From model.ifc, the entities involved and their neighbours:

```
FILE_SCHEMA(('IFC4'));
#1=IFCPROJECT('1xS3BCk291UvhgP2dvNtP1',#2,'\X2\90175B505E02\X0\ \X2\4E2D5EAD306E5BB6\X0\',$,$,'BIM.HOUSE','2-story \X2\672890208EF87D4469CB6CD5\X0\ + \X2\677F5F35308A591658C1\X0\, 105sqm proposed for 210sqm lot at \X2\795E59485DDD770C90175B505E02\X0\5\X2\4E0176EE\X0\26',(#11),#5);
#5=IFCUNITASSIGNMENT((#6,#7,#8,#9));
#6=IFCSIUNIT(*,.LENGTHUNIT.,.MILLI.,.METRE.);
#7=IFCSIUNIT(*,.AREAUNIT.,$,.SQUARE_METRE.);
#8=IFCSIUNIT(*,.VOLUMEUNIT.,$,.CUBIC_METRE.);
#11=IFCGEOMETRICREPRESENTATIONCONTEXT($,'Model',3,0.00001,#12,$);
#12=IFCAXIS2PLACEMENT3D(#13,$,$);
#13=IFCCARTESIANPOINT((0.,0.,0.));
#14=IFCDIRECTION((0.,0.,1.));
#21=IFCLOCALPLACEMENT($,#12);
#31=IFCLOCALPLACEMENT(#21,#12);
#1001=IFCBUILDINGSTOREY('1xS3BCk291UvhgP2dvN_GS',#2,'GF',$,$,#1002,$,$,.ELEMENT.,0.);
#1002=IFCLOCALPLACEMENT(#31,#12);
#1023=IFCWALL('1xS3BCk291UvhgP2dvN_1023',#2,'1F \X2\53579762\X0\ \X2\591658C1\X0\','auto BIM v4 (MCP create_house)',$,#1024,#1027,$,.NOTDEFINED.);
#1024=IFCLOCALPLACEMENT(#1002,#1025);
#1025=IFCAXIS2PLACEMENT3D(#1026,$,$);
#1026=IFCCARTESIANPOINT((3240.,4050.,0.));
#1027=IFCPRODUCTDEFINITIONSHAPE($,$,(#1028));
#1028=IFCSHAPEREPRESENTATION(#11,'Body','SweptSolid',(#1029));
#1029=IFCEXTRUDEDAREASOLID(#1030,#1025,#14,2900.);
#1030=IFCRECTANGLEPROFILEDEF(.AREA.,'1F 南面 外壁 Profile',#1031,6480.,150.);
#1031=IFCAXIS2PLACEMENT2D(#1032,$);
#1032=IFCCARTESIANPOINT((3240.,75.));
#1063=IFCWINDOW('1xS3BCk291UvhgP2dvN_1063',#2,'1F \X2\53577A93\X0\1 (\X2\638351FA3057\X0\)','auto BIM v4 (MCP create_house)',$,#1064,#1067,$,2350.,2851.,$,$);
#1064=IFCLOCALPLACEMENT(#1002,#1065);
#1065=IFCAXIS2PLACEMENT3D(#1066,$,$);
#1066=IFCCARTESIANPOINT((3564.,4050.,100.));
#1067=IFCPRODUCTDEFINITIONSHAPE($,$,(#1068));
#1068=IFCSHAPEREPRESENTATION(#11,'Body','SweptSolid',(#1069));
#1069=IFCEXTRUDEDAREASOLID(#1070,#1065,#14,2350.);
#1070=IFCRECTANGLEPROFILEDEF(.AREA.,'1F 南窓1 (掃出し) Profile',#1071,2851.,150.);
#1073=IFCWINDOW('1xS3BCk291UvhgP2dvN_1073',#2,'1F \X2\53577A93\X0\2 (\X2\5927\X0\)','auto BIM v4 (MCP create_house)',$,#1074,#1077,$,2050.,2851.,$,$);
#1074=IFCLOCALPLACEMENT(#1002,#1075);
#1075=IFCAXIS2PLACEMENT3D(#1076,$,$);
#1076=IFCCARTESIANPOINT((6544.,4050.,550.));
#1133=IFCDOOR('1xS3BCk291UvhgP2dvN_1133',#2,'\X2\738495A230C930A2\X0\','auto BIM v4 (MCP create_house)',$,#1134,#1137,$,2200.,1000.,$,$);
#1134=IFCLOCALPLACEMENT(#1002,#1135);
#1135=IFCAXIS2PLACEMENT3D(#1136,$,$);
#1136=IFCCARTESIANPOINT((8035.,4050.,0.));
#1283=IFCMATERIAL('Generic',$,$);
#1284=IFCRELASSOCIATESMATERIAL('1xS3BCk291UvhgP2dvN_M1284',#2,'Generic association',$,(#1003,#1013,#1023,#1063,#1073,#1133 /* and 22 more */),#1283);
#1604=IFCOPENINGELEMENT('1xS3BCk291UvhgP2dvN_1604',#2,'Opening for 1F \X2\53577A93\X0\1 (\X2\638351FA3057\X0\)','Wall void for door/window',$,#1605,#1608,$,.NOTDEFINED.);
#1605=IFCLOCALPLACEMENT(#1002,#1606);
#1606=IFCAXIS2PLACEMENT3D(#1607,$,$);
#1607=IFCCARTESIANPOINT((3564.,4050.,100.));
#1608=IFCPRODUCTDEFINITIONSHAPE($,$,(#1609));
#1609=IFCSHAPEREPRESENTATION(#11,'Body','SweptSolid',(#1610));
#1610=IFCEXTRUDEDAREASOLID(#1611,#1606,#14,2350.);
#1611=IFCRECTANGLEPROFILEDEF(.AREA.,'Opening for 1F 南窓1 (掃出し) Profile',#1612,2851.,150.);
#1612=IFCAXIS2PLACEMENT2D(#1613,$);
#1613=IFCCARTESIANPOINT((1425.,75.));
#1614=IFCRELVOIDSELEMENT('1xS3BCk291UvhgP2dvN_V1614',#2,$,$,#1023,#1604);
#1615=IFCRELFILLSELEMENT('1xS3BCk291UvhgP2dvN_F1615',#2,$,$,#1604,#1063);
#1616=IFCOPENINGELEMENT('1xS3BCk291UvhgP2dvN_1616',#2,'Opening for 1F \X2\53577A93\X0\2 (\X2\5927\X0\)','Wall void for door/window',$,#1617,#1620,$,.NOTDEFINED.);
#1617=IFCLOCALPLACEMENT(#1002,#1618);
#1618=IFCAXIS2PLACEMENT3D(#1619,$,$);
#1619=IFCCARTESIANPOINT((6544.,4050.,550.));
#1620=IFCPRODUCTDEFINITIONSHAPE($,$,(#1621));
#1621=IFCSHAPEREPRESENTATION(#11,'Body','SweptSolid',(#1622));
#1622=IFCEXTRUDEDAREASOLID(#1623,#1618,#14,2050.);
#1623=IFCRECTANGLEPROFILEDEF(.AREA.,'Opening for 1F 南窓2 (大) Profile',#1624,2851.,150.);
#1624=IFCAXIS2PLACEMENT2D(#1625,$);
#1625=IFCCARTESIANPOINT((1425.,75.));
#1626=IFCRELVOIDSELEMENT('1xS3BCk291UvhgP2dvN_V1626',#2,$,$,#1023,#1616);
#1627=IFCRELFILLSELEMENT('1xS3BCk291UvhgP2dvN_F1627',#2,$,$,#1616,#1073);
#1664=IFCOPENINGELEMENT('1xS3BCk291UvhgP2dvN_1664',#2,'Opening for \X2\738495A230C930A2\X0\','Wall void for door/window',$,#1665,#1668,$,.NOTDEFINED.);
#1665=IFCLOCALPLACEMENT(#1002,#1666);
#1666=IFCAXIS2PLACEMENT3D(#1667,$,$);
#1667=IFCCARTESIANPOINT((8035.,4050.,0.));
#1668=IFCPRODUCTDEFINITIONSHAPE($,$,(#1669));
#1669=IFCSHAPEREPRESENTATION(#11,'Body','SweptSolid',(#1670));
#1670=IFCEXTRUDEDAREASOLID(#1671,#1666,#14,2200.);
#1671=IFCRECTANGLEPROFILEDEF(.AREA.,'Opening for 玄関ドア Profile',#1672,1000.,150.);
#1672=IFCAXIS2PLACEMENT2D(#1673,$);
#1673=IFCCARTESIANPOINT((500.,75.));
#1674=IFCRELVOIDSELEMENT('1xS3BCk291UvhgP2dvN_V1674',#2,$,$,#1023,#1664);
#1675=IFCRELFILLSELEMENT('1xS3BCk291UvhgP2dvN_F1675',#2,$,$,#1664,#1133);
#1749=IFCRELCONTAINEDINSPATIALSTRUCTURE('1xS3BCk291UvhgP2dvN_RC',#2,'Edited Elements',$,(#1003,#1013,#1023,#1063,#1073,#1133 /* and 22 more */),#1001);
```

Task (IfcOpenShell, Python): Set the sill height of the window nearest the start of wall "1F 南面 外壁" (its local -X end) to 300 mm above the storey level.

```python
import numpy as np
import ifcopenshell
import ifcopenshell.api.geometry
import ifcopenshell.geom
import ifcopenshell.util.element
import ifcopenshell.util.placement
import ifcopenshell.util.shape
import ifcopenshell.util.unit

model = ifcopenshell.open("model.ifc")
unit_scale = ifcopenshell.util.unit.calculate_unit_scale(model)

window = model.by_guid("1xS3BCk291UvhgP2dvN_1063")
opening = window.FillsVoids[0].RelatingOpeningElement
storey = ifcopenshell.util.element.get_container(window, ifc_class="IfcBuildingStorey")
level = ifcopenshell.util.placement.get_local_placement(storey.ObjectPlacement)[2, 3]

# The opening's origin need not be at the sill, so measure its lowest point.
shape = ifcopenshell.geom.create_shape(ifcopenshell.geom.settings(), opening)
bottom = ifcopenshell.util.shape.get_shape_bottom_elevation(shape, shape.geometry) / unit_scale
dz = level + 0.3 / unit_scale - bottom

shift = np.array([0.0, 0.0, dz])
# The window is not placed relative to its opening, so move both.
for product in (opening, window):
    matrix = ifcopenshell.util.placement.get_local_placement(product.ObjectPlacement)
    matrix[:3, 3] += shift
    ifcopenshell.api.geometry.edit_object_placement(model, product=product, matrix=matrix, is_si=False)

print(f"moved by {dz * unit_scale:+.3f} m")

model.write("model_v2.ifc")
```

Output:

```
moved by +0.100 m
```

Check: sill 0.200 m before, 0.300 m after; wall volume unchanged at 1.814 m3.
